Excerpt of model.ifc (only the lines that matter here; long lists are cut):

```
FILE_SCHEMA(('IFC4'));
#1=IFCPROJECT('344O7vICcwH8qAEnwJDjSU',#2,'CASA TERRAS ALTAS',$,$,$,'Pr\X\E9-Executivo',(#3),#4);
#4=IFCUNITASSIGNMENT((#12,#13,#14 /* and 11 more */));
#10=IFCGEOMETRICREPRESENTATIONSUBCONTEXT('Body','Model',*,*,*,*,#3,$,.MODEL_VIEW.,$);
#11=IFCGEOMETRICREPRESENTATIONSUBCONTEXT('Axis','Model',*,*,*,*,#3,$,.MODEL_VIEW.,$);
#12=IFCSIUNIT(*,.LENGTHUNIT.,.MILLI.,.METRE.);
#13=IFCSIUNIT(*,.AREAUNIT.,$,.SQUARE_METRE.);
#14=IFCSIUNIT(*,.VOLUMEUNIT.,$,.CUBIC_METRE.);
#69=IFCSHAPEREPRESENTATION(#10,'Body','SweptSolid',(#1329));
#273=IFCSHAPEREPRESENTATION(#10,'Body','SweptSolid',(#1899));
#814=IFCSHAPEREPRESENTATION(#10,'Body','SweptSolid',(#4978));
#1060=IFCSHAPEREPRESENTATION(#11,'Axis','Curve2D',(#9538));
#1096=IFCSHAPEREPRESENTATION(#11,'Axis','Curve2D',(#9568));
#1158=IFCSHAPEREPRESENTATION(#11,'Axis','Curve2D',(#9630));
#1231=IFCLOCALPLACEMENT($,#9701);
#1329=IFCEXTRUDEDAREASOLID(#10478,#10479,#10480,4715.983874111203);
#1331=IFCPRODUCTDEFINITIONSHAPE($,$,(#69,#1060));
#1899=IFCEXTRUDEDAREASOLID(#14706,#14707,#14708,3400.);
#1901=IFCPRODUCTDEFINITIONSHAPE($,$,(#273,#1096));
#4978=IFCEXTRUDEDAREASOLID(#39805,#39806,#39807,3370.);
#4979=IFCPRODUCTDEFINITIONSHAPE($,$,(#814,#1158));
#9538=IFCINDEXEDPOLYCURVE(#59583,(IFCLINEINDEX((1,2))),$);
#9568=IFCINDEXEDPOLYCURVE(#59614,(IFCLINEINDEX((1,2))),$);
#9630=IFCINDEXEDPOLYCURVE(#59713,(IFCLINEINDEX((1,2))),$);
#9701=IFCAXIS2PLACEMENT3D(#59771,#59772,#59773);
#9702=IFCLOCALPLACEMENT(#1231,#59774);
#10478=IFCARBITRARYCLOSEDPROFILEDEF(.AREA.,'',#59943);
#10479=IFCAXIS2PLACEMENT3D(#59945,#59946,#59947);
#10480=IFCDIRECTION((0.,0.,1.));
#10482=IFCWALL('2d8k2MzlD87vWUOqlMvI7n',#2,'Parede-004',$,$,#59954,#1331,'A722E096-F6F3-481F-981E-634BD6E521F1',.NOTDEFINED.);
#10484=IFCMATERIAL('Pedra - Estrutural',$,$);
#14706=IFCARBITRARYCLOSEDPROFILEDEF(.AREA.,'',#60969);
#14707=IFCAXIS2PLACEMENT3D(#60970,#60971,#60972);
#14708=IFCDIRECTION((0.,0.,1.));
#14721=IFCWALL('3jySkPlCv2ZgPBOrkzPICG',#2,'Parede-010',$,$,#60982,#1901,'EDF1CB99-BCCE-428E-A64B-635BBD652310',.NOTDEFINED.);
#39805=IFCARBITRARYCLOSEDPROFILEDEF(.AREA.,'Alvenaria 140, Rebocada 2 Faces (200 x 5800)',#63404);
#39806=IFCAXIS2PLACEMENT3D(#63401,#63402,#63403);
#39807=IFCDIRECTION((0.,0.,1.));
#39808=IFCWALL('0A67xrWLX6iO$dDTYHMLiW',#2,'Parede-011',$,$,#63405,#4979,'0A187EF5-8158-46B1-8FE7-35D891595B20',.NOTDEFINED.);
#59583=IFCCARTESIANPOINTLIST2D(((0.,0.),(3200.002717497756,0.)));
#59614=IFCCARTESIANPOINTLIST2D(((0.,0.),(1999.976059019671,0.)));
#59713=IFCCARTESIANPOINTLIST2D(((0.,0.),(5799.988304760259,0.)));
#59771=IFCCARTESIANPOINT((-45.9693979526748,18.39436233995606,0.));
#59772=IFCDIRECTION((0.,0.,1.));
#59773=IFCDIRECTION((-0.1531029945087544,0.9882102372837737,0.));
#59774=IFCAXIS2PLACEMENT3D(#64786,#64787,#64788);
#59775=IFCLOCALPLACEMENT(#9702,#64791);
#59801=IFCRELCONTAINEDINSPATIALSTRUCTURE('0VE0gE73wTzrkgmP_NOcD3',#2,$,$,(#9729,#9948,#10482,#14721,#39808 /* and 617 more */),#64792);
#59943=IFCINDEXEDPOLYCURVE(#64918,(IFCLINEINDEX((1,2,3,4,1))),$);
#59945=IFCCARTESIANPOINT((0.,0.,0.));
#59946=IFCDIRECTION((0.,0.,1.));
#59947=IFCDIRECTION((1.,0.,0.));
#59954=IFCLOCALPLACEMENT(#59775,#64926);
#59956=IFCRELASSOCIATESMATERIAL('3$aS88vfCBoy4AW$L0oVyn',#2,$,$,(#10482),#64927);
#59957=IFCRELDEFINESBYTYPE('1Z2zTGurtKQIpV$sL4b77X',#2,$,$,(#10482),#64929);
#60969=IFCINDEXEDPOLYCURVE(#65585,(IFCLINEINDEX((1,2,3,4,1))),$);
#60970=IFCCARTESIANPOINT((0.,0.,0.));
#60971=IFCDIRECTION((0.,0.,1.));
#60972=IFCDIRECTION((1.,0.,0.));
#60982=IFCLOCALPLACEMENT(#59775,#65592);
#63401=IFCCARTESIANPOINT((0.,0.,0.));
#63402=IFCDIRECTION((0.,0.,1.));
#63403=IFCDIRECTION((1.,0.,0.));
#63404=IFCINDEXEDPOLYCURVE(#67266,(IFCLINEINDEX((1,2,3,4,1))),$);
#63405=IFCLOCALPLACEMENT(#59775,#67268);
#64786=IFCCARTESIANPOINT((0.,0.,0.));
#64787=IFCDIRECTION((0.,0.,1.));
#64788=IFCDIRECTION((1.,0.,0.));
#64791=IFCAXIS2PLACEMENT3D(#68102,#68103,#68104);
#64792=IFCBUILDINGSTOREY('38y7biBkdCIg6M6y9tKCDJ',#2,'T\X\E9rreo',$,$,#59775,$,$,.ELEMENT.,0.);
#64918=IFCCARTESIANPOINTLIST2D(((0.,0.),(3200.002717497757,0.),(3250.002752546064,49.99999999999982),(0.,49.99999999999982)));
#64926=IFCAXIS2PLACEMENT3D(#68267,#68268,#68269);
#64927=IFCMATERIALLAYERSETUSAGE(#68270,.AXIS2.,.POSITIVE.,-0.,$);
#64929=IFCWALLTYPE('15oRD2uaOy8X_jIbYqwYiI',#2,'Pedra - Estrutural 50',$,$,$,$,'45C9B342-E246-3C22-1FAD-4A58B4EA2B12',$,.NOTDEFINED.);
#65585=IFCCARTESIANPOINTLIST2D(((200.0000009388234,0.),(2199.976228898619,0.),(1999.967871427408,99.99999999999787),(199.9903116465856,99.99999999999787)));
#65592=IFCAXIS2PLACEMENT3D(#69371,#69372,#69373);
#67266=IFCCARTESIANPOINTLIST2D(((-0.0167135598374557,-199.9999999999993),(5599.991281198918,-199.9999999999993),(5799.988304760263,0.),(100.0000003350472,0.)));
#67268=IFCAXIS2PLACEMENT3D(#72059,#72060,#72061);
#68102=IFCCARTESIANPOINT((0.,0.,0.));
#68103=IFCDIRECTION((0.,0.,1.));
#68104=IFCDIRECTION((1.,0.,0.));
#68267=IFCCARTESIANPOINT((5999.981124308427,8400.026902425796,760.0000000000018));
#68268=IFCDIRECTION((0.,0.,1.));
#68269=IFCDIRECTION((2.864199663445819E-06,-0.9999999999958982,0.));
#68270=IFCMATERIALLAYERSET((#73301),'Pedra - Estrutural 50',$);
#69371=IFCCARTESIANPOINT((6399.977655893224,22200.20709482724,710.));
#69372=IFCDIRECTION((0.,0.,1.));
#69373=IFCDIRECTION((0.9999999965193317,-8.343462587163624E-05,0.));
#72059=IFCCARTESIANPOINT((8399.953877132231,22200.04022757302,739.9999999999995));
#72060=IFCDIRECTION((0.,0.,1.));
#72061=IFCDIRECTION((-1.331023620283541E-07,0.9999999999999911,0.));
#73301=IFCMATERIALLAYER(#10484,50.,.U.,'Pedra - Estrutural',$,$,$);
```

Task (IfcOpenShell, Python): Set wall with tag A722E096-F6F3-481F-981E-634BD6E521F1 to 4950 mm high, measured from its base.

```python
import ifcopenshell
import ifcopenshell.geom
import ifcopenshell.util.representation
import ifcopenshell.util.shape
import ifcopenshell.util.unit

model = ifcopenshell.open("model.ifc")
unit_scale = ifcopenshell.util.unit.calculate_unit_scale(model)
settings = ifcopenshell.geom.settings()


def volume(element):
    """Net volume in cubic metres, openings subtracted."""
    shape = ifcopenshell.geom.create_shape(settings, element)
    return ifcopenshell.util.shape.get_volume(shape.geometry)


wall = model.by_guid("2d8k2MzlD87vWUOqlMvI7n")
before = volume(wall)

body = ifcopenshell.util.representation.get_representation(wall, "Model", "Body")
solid = body.Items[0]
old_height = solid.Depth
solid.Depth = 4.95 / unit_scale
after = volume(wall)

print(f"height {old_height:g} -> {solid.Depth:g}, volume {before:.3f} -> {after:.3f} m3")

model.write("model_updated.ifc")
```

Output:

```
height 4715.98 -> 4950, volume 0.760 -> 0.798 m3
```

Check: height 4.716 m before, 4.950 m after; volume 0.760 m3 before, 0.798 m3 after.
